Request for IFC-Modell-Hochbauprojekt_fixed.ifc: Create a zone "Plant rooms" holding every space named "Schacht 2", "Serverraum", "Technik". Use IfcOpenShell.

First a look at what the model holds.

```python
import ifcopenshell

model = ifcopenshell.open("IFC-Modell-Hochbauprojekt_fixed.ifc")
print(model.schema)
seen = {}
for space in model.by_type("IfcSpace"):
    seen[space.LongName] = seen.get(space.LongName, 0) + 1
for name, count in sorted(seen.items(), key=str):
    print(count, "x", name)
print("zones:", [z.Name for z in model.by_type("IfcZone")][:20])
```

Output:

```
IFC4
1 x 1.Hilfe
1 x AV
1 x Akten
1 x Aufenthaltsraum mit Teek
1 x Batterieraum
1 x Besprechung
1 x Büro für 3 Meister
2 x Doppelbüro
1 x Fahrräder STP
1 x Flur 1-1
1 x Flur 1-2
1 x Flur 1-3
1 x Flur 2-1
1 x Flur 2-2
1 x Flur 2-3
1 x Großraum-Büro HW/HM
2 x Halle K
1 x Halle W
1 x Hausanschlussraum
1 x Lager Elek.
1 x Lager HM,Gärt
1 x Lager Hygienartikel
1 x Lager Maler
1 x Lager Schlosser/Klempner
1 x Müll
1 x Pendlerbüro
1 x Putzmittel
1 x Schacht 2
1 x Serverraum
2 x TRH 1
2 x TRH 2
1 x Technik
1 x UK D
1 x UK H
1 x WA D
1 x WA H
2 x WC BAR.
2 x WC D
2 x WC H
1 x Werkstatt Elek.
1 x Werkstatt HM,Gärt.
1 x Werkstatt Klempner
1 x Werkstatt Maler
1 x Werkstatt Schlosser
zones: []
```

```python
import ifcopenshell
import ifcopenshell.api.group
import ifcopenshell.api.root

model = ifcopenshell.open("IFC-Modell-Hochbauprojekt_fixed.ifc")

names = {"Schacht 2", "Serverraum", "Technik"}
spaces = [s for s in model.by_type("IfcSpace") if s.LongName in names]

zone = ifcopenshell.api.root.create_entity(model, ifc_class="IfcZone", name="Plant rooms")
ifcopenshell.api.group.assign_group(model, products=spaces, group=zone)
print(len(spaces), "spaces in", zone.Name)

model.write("IFC-Modell-Hochbauprojekt_fixed_updated.ifc")
```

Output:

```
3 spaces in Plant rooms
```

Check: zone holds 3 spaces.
